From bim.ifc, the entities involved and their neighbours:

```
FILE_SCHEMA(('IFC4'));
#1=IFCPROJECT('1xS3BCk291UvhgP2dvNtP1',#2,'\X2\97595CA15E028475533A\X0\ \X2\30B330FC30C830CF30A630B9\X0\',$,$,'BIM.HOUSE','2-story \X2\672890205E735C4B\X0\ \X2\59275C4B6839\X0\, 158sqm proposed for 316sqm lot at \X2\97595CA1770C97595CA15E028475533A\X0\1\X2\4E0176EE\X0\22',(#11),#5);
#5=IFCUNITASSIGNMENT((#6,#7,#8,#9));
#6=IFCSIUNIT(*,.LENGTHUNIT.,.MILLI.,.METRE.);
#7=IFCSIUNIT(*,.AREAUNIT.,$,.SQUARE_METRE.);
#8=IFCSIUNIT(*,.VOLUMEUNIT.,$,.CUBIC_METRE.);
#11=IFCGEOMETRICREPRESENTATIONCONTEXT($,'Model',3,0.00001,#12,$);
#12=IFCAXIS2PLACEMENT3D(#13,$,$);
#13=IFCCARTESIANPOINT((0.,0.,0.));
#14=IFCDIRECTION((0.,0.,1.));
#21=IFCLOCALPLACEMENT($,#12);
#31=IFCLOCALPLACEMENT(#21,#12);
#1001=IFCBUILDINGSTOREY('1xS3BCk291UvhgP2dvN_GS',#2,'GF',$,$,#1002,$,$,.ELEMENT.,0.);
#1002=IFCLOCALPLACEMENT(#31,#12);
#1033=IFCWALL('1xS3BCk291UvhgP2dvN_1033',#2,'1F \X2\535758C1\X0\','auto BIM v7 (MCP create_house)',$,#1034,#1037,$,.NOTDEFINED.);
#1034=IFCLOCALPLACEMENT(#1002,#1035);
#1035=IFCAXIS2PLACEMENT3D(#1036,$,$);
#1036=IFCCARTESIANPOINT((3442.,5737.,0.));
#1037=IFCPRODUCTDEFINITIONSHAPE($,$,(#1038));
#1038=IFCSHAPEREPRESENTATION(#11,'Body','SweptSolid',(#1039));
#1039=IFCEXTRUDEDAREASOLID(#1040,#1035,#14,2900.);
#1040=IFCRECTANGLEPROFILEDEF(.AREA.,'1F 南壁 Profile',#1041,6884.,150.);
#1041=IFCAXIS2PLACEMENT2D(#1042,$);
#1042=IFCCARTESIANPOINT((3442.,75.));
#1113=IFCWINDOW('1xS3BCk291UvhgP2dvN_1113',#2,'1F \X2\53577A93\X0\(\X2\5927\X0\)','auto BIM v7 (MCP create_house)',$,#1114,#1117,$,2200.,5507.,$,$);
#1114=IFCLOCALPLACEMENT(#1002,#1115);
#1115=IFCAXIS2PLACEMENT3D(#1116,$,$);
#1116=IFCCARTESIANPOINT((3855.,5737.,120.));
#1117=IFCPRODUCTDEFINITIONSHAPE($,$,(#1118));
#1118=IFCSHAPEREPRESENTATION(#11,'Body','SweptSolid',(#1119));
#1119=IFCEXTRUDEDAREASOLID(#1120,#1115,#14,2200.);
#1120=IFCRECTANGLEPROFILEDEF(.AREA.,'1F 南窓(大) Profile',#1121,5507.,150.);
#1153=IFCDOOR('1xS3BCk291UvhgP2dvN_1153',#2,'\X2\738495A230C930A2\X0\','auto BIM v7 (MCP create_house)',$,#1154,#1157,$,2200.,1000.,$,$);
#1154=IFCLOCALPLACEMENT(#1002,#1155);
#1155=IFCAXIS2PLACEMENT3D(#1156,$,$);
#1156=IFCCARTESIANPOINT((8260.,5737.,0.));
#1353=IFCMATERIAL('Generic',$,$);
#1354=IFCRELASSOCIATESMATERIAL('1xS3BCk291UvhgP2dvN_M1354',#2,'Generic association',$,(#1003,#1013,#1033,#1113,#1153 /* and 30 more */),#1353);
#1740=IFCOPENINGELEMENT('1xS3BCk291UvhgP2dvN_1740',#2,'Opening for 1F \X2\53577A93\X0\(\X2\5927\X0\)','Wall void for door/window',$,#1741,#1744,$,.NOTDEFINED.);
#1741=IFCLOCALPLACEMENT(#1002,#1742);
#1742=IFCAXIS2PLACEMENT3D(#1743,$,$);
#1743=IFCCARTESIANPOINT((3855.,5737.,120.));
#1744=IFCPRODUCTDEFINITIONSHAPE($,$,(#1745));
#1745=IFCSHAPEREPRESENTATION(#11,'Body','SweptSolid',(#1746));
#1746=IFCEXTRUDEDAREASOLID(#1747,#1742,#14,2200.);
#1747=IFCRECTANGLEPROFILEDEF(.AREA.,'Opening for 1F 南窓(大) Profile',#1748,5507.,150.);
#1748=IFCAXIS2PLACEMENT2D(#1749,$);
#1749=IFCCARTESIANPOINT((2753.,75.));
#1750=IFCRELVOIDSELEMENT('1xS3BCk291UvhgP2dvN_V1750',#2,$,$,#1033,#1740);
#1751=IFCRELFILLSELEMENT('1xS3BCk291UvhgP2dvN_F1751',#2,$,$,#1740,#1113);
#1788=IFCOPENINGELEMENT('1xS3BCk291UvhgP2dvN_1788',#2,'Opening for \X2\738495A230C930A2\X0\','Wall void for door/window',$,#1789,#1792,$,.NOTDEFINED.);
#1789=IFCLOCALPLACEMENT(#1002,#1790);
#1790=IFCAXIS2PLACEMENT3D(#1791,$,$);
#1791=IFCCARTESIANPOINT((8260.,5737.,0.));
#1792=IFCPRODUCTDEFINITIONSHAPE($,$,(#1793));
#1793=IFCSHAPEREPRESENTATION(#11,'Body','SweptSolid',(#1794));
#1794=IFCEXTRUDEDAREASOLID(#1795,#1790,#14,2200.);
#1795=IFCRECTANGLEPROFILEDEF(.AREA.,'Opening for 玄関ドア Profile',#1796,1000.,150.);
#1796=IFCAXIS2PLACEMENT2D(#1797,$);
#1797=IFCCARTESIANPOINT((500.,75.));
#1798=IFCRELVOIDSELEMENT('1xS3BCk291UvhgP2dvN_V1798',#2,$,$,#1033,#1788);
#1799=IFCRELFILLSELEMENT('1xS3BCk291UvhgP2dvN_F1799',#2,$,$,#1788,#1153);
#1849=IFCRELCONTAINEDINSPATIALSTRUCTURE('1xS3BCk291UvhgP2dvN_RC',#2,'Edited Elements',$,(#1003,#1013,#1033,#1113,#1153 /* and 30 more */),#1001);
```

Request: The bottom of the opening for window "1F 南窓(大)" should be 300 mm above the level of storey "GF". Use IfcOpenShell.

```python
import numpy as np
import ifcopenshell
import ifcopenshell.api.geometry
import ifcopenshell.geom
import ifcopenshell.util.element
import ifcopenshell.util.placement
import ifcopenshell.util.shape
import ifcopenshell.util.unit

model = ifcopenshell.open("bim.ifc")
unit_scale = ifcopenshell.util.unit.calculate_unit_scale(model)

window = model.by_id(1113)
opening = window.FillsVoids[0].RelatingOpeningElement
storey = ifcopenshell.util.element.get_container(window, ifc_class="IfcBuildingStorey")
level = ifcopenshell.util.placement.get_local_placement(storey.ObjectPlacement)[2, 3]

# The opening's origin need not be at the sill, so measure its lowest point.
shape = ifcopenshell.geom.create_shape(ifcopenshell.geom.settings(), opening)
bottom = ifcopenshell.util.shape.get_shape_bottom_elevation(shape, shape.geometry) / unit_scale
dz = level + 0.3 / unit_scale - bottom

shift = np.array([0.0, 0.0, dz])
# The window is not placed relative to its opening, so move both.
for product in (opening, window):
    matrix = ifcopenshell.util.placement.get_local_placement(product.ObjectPlacement)
    matrix[:3, 3] += shift
    ifcopenshell.api.geometry.edit_object_placement(model, product=product, matrix=matrix, is_si=False)

print(f"moved by {dz * unit_scale:+.3f} m")

model.write("bim_v2.ifc")
```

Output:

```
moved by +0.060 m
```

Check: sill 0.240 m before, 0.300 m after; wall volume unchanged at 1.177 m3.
